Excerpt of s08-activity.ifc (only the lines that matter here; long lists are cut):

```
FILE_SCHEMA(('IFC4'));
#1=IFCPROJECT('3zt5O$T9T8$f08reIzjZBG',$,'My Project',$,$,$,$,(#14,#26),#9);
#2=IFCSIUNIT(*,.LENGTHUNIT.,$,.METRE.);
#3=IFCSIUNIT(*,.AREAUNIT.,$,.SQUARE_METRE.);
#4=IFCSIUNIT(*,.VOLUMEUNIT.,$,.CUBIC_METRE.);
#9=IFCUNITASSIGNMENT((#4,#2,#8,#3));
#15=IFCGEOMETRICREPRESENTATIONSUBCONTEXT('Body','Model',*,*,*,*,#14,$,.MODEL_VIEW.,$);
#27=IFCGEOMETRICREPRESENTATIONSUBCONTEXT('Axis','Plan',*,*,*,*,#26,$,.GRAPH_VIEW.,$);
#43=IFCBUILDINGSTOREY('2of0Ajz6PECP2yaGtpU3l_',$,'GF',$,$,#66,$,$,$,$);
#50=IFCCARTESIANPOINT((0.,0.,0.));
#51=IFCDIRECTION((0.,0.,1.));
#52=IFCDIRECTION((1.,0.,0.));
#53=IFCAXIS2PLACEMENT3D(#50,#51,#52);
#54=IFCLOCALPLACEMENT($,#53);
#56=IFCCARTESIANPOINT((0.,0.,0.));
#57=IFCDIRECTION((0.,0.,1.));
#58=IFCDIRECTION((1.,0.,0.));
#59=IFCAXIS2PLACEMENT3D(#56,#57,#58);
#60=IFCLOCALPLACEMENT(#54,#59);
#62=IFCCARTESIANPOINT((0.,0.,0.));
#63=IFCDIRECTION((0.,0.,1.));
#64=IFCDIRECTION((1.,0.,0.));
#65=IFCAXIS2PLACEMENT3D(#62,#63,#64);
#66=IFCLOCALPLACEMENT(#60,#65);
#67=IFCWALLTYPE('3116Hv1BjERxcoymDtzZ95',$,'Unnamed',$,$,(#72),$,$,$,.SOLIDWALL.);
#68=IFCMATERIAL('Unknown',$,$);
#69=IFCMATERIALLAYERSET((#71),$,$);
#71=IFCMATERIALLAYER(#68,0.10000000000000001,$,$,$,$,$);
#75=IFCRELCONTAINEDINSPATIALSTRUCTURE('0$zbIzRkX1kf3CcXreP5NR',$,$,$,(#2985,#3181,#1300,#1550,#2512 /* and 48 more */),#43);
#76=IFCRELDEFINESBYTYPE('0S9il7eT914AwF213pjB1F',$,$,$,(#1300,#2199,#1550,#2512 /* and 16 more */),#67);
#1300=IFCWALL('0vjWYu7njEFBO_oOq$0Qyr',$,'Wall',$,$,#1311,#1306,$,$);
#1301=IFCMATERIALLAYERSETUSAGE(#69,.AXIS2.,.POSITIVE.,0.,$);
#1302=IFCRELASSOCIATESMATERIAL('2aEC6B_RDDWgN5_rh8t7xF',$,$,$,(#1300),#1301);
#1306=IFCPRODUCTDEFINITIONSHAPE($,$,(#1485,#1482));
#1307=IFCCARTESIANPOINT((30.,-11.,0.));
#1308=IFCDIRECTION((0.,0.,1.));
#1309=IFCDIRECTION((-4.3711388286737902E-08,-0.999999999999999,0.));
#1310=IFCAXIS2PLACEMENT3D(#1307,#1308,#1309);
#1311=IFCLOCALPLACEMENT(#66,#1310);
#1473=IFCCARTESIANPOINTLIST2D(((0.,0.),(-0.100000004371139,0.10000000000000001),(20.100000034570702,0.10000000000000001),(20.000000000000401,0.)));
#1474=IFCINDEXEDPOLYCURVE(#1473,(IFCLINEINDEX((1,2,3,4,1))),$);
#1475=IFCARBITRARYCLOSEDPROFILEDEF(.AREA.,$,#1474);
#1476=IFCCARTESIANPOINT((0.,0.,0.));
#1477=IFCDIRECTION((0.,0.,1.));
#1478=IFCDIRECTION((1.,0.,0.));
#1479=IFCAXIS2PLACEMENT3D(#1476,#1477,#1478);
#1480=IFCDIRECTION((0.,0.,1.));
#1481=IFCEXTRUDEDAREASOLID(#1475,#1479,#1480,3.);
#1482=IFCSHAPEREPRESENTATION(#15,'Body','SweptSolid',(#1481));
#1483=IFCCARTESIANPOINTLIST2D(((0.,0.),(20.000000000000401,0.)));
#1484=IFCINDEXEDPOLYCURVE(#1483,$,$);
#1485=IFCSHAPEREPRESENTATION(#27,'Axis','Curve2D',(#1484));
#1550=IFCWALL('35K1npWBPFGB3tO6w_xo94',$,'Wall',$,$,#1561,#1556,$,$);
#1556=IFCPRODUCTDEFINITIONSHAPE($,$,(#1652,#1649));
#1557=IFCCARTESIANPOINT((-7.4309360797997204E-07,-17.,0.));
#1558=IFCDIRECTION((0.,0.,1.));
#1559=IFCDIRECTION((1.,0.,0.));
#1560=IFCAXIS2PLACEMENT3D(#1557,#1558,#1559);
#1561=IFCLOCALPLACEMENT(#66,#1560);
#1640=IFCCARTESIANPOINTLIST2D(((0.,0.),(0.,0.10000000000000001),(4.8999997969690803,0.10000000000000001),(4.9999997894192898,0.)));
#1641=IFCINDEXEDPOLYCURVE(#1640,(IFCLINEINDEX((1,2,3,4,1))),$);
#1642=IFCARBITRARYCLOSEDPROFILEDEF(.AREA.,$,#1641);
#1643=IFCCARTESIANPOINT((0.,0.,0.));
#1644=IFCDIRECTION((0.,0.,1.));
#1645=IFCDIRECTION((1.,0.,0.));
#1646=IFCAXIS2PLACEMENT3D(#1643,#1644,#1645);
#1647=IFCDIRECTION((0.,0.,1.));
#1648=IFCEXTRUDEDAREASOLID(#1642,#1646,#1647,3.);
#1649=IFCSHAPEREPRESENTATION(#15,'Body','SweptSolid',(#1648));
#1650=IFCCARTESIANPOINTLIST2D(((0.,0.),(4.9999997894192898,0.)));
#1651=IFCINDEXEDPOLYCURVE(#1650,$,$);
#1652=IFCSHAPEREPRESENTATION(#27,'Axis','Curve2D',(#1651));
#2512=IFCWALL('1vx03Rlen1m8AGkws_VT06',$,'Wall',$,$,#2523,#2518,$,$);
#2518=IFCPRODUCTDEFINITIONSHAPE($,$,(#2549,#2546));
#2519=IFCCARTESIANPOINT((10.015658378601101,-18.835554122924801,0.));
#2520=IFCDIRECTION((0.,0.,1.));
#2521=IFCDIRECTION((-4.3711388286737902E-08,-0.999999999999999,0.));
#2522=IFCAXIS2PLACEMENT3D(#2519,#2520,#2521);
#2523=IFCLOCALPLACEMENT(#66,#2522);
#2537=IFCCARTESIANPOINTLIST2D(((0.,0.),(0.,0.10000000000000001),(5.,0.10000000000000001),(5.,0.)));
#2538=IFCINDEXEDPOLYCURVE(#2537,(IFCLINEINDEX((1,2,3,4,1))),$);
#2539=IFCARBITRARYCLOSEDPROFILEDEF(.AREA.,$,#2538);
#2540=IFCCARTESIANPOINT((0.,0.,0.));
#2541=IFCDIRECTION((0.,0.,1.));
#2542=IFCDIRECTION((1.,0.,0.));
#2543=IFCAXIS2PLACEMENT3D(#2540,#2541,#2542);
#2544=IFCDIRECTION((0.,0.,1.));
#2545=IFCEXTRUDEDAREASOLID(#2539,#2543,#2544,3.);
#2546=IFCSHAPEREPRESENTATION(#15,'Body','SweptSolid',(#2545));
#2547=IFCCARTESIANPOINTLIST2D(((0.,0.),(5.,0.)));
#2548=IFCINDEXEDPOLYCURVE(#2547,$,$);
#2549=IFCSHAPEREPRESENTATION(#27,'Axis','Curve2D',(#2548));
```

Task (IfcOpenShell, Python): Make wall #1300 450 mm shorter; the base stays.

```python
import ifcopenshell
import ifcopenshell.geom
import ifcopenshell.util.representation
import ifcopenshell.util.shape
import ifcopenshell.util.unit

model = ifcopenshell.open("s08-activity.ifc")
unit_scale = ifcopenshell.util.unit.calculate_unit_scale(model)
settings = ifcopenshell.geom.settings()


def volume(element):
    """Net volume in cubic metres, openings subtracted."""
    shape = ifcopenshell.geom.create_shape(settings, element)
    return ifcopenshell.util.shape.get_volume(shape.geometry)


wall = model.by_id(1300)
before = volume(wall)

body = ifcopenshell.util.representation.get_representation(wall, "Model", "Body")
solid = body.Items[0]
old_height = solid.Depth
solid.Depth -= 0.45 / unit_scale
after = volume(wall)

print(f"height {old_height:g} -> {solid.Depth:g}, volume {before:.3f} -> {after:.3f} m3")

model.write("s08-activity_rev.ifc")
```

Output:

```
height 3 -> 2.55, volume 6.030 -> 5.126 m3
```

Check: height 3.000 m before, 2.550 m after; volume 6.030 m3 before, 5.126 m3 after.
